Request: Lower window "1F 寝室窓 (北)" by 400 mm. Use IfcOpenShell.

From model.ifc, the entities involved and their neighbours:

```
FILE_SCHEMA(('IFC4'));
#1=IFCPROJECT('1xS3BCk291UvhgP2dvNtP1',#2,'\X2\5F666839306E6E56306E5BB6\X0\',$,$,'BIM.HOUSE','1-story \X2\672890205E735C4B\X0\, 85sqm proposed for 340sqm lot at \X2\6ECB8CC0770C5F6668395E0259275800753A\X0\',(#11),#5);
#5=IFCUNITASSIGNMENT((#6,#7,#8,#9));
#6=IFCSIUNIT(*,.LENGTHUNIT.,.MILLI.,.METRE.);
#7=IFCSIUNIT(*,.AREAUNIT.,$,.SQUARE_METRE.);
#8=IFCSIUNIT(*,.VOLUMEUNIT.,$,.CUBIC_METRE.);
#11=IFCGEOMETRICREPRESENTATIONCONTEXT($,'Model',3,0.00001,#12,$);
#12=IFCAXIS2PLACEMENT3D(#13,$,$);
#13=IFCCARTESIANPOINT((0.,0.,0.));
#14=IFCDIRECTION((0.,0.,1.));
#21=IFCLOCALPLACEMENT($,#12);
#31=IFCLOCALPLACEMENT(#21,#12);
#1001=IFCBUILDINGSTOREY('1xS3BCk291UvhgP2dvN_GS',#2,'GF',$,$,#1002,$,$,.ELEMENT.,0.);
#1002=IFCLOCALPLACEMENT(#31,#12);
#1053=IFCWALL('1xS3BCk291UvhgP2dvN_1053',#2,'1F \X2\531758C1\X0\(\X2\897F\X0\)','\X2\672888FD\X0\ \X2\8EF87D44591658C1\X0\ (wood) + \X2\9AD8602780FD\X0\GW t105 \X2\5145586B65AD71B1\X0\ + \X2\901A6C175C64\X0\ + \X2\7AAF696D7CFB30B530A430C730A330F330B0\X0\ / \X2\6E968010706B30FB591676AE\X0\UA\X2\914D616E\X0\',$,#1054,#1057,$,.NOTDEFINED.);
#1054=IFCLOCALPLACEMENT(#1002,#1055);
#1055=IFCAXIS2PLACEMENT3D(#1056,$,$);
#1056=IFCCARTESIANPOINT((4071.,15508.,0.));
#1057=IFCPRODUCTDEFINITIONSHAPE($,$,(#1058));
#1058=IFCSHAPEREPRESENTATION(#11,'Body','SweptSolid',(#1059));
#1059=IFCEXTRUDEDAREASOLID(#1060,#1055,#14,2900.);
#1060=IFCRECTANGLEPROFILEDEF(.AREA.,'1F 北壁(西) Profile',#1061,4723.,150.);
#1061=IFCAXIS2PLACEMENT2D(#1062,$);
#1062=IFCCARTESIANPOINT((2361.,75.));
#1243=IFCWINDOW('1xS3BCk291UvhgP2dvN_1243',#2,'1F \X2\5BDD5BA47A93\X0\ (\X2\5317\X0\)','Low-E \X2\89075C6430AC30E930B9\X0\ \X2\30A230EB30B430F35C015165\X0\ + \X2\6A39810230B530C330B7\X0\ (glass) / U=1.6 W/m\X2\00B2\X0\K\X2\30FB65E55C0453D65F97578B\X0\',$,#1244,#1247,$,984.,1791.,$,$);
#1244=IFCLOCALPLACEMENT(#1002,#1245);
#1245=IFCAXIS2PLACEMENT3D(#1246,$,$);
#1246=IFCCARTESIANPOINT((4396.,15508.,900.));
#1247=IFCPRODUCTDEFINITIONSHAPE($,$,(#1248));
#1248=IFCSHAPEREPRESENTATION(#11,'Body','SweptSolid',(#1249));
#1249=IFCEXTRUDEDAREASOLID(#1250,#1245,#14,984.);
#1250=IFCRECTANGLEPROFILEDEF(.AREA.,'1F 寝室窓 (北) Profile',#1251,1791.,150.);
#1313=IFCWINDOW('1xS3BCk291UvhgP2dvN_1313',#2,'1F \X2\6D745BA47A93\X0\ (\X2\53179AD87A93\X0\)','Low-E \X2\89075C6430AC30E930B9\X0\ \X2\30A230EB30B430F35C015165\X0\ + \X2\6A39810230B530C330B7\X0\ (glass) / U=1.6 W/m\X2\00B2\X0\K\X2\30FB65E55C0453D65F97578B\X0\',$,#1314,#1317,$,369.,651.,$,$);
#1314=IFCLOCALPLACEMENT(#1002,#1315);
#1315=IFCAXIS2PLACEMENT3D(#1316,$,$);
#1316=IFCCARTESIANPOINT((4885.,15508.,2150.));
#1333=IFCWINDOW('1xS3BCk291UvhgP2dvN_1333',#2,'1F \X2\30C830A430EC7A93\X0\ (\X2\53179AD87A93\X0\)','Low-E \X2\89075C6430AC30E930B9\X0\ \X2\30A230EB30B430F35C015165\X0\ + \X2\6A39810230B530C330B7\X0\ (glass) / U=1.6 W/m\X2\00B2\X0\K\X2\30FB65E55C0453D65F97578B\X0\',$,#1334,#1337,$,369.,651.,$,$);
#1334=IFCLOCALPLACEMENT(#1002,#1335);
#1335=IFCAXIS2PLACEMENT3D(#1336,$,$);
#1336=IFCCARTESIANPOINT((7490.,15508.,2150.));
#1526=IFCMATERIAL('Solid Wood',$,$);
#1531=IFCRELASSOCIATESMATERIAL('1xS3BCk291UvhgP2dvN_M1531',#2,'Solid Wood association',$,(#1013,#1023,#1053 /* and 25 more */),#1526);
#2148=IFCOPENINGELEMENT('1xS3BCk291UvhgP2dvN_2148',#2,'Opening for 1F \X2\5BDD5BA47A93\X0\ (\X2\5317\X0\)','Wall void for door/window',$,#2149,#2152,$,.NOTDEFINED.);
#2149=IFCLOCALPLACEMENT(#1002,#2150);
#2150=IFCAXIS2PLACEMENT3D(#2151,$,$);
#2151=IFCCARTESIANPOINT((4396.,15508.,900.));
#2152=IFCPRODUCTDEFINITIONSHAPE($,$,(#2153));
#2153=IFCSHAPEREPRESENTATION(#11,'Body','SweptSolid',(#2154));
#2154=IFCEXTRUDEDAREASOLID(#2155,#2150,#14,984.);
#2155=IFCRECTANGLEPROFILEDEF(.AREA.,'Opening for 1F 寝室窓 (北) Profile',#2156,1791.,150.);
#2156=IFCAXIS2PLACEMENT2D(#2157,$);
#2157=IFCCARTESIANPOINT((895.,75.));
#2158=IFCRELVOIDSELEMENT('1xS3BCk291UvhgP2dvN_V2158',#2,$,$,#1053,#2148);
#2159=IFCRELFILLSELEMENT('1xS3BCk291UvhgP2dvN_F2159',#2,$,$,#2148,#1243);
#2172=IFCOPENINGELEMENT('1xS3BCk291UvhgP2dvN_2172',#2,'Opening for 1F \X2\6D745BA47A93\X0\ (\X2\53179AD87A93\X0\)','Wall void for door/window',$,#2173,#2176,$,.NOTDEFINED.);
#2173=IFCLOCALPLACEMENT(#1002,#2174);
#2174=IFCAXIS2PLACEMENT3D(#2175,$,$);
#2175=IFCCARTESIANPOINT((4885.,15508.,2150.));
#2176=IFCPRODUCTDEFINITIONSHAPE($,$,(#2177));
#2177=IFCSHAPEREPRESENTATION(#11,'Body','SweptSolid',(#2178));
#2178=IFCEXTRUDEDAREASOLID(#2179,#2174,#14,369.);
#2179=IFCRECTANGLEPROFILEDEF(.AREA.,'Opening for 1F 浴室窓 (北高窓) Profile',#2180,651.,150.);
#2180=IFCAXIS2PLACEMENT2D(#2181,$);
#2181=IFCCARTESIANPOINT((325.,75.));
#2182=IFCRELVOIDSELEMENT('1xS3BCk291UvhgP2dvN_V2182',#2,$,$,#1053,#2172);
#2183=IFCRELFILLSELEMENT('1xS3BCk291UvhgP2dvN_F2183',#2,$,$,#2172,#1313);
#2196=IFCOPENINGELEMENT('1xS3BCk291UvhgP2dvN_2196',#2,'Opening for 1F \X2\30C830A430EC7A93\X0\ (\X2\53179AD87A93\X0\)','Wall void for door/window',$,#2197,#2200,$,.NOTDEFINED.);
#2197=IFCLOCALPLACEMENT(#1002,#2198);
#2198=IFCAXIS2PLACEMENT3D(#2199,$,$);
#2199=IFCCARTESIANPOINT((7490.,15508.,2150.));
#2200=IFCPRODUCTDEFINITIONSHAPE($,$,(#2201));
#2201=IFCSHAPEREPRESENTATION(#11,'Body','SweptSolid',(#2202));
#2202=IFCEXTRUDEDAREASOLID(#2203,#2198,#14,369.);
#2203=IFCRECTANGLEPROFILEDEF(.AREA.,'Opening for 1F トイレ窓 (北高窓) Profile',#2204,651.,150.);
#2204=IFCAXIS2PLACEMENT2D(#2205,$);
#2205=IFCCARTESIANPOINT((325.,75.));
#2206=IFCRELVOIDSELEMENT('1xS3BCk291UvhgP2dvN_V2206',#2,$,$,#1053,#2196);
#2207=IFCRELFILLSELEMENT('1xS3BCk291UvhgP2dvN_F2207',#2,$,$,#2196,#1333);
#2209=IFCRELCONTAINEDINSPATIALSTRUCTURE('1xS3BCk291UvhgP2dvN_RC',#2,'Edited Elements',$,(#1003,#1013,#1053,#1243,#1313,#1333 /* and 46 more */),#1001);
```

```python
import numpy as np
import ifcopenshell
import ifcopenshell.api.geometry
import ifcopenshell.util.placement
import ifcopenshell.util.unit

model = ifcopenshell.open("model.ifc")
unit_scale = ifcopenshell.util.unit.calculate_unit_scale(model)

window = model.by_guid("1xS3BCk291UvhgP2dvN_1243")
opening = window.FillsVoids[0].RelatingOpeningElement
dz = -0.4 / unit_scale

shift = np.array([0.0, 0.0, dz])
# The window is not placed relative to its opening, so move both.
for product in (opening, window):
    matrix = ifcopenshell.util.placement.get_local_placement(product.ObjectPlacement)
    matrix[:3, 3] += shift
    ifcopenshell.api.geometry.edit_object_placement(model, product=product, matrix=matrix, is_si=False)

print(f"moved by {dz * unit_scale:+.3f} m")

model.write("model_rev.ifc")
```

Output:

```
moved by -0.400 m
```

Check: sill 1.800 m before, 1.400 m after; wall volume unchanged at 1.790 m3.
